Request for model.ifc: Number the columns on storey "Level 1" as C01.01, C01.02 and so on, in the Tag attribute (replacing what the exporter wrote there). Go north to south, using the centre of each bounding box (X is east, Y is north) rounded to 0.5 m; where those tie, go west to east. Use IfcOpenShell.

First a look at what the model holds.

```python
import ifcopenshell
import ifcopenshell.util.element
import ifcopenshell.util.placement

model = ifcopenshell.open("model.ifc")
print(model.schema)
storey = next(s for s in model.by_type("IfcBuildingStorey") if s.Name == "Level 1")
columns = [e for e in ifcopenshell.util.element.get_decomposition(storey) if e.is_a("IfcColumn")]
for e in sorted(columns, key=lambda e: e.id()):
    origin = ifcopenshell.util.placement.get_local_placement(e.ObjectPlacement)[:3, 3]
    print(e.id(), e.Tag, e.Name, origin.round(2) + 0.0, sep=" | ")
```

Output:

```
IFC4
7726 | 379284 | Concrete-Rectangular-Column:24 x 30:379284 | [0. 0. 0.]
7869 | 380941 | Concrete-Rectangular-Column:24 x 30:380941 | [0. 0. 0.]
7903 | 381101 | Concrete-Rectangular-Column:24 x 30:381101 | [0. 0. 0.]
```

```python
import ifcopenshell
import ifcopenshell.geom
import ifcopenshell.util.element
import ifcopenshell.util.shape

model = ifcopenshell.open("model.ifc")
settings = ifcopenshell.geom.settings()
settings.set("use-world-coords", True)


def centre(element):
    shape = ifcopenshell.geom.create_shape(settings, element)
    return ifcopenshell.util.shape.get_bbox_centroid(shape.geometry)


storey = next(s for s in model.by_type("IfcBuildingStorey") if s.Name == "Level 1")
columns = [e for e in ifcopenshell.util.element.get_decomposition(storey) if e.is_a("IfcColumn")]

# Insertion points can sit at a corner or the storey origin, so sort by the geometry (in metres).
centres = {e: centre(e) for e in columns}
columns.sort(key=lambda e: (-round(centres[e][1] / 0.5), centres[e][0]))

for i, e in enumerate(columns, start=1):
    number = f"C01.{i:02d}"
    e.Tag = number
    print(e.id(), number)

model.write("model_updated.ifc")
```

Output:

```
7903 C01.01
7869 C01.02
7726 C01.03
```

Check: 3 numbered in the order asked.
